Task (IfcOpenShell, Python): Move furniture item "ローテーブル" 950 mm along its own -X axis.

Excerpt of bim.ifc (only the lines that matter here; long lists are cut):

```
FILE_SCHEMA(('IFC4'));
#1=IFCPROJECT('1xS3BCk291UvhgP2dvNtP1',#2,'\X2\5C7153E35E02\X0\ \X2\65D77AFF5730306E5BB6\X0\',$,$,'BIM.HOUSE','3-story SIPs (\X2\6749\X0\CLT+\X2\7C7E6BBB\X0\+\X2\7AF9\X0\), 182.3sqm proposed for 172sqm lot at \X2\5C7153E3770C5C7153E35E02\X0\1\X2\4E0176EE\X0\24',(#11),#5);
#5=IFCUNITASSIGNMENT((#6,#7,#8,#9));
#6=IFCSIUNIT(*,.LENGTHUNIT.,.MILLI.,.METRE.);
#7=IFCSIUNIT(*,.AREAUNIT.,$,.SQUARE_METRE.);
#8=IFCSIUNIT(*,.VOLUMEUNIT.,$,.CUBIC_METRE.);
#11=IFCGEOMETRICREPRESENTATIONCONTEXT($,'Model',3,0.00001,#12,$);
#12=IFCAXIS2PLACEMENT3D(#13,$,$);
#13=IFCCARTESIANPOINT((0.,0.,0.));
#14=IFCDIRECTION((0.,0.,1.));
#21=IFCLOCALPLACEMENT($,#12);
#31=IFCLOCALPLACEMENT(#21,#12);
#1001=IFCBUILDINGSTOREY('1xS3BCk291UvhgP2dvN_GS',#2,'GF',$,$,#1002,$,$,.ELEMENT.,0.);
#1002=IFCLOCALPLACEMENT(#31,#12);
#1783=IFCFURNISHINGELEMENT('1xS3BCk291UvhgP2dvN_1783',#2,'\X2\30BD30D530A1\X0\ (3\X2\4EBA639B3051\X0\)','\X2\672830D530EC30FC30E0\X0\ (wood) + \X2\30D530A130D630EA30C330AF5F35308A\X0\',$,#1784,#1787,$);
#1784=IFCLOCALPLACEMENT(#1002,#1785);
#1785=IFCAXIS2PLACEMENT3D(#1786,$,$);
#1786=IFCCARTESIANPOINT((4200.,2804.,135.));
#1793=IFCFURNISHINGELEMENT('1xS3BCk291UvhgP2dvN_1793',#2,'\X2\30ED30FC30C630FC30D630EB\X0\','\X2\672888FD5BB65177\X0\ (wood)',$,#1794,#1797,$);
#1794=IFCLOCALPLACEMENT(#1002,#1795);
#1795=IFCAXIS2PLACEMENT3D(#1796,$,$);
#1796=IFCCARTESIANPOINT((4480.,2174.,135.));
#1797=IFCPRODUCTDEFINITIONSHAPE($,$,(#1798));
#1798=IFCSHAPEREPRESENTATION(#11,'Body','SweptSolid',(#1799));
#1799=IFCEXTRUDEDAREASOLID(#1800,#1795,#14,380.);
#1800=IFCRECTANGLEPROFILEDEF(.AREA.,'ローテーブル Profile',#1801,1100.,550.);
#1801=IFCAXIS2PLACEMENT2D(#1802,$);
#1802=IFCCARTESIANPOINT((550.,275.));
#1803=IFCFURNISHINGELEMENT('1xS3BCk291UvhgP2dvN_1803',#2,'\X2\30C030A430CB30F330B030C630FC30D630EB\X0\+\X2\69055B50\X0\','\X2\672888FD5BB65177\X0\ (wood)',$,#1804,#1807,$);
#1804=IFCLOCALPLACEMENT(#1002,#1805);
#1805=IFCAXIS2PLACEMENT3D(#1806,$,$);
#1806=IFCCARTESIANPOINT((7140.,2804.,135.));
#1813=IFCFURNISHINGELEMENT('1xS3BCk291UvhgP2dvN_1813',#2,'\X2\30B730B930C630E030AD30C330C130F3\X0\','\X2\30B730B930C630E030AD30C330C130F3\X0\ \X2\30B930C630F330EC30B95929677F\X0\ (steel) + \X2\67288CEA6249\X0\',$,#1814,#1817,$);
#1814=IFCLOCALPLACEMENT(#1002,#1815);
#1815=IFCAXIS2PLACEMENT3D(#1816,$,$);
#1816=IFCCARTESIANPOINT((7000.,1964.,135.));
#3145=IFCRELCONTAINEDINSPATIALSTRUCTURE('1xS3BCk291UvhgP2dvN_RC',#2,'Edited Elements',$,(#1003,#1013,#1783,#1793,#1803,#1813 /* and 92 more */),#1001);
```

```python
import ifcopenshell
import ifcopenshell.api.geometry
import ifcopenshell.util.placement
import ifcopenshell.util.unit

model = ifcopenshell.open("bim.ifc")
unit_scale = ifcopenshell.util.unit.calculate_unit_scale(model)

item = model.by_guid("1xS3BCk291UvhgP2dvN_1793")
matrix = ifcopenshell.util.placement.get_local_placement(item.ObjectPlacement)
matrix[:3, 3] -= matrix[:3, 0] * 0.95 / unit_scale
ifcopenshell.api.geometry.edit_object_placement(model, product=item, matrix=matrix, is_si=False)

print(ifcopenshell.util.placement.get_local_placement(item.ObjectPlacement).round(3) + 0.0)

model.write("bim-out.ifc")
```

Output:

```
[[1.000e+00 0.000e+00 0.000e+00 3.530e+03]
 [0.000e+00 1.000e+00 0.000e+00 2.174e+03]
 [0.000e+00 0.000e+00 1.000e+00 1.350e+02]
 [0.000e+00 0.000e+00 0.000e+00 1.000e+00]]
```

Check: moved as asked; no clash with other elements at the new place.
